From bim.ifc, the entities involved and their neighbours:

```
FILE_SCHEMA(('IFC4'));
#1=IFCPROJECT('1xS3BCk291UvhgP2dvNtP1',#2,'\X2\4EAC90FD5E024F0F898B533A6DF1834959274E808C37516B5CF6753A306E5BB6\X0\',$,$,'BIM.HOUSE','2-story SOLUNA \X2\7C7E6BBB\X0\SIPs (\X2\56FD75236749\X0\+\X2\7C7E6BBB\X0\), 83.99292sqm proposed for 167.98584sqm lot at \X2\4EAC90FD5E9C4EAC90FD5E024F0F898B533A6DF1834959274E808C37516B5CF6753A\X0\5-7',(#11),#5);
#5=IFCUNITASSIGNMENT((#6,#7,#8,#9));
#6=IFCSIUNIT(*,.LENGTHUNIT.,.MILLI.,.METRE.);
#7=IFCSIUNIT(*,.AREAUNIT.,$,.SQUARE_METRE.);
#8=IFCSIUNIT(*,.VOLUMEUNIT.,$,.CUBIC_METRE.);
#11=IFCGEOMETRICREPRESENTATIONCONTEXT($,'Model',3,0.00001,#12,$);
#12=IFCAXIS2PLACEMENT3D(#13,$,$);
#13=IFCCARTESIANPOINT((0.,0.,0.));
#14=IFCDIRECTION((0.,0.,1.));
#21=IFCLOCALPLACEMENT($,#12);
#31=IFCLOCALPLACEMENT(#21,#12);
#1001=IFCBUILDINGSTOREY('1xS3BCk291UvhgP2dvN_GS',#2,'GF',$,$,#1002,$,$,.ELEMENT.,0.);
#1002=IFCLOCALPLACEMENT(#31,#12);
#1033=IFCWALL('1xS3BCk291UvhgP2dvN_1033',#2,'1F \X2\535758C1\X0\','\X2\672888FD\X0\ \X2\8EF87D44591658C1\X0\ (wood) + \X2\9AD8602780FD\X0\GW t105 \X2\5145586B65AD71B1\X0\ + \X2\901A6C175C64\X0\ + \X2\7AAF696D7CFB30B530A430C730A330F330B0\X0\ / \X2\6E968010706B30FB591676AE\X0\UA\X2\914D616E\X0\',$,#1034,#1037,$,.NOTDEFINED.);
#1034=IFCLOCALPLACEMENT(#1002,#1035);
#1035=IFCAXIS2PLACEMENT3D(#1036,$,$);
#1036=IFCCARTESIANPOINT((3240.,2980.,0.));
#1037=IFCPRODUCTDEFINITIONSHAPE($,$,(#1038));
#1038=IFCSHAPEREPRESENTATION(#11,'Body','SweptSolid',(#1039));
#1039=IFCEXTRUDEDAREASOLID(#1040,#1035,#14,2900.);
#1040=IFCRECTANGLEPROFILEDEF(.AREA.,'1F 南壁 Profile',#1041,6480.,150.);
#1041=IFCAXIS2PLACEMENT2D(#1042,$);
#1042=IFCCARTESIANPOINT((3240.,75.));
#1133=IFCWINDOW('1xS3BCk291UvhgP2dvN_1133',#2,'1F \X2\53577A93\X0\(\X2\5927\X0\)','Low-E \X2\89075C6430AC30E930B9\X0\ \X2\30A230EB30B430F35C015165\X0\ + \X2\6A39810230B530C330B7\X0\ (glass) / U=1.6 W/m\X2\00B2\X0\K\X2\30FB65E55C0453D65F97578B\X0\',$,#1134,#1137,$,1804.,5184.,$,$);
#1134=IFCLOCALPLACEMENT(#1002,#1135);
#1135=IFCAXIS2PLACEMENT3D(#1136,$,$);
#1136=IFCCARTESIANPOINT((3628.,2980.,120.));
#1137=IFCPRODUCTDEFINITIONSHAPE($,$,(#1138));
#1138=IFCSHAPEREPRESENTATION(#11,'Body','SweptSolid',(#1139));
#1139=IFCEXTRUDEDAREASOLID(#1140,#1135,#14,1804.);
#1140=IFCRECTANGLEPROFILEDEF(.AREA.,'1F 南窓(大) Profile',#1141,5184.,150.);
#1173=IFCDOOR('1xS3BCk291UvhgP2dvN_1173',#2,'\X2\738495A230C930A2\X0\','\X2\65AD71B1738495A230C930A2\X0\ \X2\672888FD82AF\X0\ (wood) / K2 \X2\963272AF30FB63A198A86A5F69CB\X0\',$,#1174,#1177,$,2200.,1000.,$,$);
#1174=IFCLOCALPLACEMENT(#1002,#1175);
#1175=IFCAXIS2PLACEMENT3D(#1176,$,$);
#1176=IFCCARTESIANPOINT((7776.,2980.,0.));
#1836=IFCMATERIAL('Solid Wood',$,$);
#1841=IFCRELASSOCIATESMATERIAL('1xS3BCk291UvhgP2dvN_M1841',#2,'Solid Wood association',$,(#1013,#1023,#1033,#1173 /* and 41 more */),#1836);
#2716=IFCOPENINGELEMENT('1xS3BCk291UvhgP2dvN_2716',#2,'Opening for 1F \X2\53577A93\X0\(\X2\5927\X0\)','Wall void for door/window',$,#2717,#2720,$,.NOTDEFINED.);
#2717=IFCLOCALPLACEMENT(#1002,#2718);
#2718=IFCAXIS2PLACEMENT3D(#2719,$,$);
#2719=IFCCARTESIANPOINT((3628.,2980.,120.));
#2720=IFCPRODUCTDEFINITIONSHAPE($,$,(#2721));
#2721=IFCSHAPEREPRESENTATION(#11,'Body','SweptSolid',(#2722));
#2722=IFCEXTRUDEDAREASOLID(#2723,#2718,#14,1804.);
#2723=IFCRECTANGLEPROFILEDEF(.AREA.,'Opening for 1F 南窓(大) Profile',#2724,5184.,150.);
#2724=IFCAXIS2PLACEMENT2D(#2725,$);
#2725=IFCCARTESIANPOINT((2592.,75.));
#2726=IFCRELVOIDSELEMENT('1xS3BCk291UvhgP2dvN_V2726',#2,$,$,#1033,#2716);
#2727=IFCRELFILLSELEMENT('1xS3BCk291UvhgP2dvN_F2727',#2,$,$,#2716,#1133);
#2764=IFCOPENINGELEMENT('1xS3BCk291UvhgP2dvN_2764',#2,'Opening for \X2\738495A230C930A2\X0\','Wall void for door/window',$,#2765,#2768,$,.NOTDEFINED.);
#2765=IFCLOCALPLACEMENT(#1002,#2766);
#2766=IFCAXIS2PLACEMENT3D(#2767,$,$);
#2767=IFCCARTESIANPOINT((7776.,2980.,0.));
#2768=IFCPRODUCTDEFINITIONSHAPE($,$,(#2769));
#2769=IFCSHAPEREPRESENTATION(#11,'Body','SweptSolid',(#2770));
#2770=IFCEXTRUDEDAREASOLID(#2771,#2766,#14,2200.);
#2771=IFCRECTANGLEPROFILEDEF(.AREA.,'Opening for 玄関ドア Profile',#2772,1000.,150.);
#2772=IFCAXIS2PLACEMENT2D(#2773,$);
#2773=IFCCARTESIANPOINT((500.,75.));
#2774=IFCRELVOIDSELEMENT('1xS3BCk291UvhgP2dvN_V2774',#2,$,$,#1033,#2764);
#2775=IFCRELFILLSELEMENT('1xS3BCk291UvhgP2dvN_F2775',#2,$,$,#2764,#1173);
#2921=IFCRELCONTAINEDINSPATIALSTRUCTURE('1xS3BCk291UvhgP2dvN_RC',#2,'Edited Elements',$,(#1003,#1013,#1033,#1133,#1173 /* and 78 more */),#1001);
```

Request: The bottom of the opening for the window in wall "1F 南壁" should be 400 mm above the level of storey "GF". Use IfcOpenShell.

```python
import numpy as np
import ifcopenshell
import ifcopenshell.api.geometry
import ifcopenshell.geom
import ifcopenshell.util.element
import ifcopenshell.util.placement
import ifcopenshell.util.shape
import ifcopenshell.util.unit

model = ifcopenshell.open("bim.ifc")
unit_scale = ifcopenshell.util.unit.calculate_unit_scale(model)

window = model.by_id(1133)
opening = window.FillsVoids[0].RelatingOpeningElement
storey = ifcopenshell.util.element.get_container(window, ifc_class="IfcBuildingStorey")
level = ifcopenshell.util.placement.get_local_placement(storey.ObjectPlacement)[2, 3]

# The opening's origin need not be at the sill, so measure its lowest point.
shape = ifcopenshell.geom.create_shape(ifcopenshell.geom.settings(), opening)
bottom = ifcopenshell.util.shape.get_shape_bottom_elevation(shape, shape.geometry) / unit_scale
dz = level + 400.0 - bottom

shift = np.array([0.0, 0.0, dz])
# The window is not placed relative to its opening, so move both.
for product in (opening, window):
    matrix = ifcopenshell.util.placement.get_local_placement(product.ObjectPlacement)
    matrix[:3, 3] += shift
    ifcopenshell.api.geometry.edit_object_placement(model, product=product, matrix=matrix, is_si=False)

print(f"moved by {dz * unit_scale:+.3f} m")

model.write("bim-out.ifc")
```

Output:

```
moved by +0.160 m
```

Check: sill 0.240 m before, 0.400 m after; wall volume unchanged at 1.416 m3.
